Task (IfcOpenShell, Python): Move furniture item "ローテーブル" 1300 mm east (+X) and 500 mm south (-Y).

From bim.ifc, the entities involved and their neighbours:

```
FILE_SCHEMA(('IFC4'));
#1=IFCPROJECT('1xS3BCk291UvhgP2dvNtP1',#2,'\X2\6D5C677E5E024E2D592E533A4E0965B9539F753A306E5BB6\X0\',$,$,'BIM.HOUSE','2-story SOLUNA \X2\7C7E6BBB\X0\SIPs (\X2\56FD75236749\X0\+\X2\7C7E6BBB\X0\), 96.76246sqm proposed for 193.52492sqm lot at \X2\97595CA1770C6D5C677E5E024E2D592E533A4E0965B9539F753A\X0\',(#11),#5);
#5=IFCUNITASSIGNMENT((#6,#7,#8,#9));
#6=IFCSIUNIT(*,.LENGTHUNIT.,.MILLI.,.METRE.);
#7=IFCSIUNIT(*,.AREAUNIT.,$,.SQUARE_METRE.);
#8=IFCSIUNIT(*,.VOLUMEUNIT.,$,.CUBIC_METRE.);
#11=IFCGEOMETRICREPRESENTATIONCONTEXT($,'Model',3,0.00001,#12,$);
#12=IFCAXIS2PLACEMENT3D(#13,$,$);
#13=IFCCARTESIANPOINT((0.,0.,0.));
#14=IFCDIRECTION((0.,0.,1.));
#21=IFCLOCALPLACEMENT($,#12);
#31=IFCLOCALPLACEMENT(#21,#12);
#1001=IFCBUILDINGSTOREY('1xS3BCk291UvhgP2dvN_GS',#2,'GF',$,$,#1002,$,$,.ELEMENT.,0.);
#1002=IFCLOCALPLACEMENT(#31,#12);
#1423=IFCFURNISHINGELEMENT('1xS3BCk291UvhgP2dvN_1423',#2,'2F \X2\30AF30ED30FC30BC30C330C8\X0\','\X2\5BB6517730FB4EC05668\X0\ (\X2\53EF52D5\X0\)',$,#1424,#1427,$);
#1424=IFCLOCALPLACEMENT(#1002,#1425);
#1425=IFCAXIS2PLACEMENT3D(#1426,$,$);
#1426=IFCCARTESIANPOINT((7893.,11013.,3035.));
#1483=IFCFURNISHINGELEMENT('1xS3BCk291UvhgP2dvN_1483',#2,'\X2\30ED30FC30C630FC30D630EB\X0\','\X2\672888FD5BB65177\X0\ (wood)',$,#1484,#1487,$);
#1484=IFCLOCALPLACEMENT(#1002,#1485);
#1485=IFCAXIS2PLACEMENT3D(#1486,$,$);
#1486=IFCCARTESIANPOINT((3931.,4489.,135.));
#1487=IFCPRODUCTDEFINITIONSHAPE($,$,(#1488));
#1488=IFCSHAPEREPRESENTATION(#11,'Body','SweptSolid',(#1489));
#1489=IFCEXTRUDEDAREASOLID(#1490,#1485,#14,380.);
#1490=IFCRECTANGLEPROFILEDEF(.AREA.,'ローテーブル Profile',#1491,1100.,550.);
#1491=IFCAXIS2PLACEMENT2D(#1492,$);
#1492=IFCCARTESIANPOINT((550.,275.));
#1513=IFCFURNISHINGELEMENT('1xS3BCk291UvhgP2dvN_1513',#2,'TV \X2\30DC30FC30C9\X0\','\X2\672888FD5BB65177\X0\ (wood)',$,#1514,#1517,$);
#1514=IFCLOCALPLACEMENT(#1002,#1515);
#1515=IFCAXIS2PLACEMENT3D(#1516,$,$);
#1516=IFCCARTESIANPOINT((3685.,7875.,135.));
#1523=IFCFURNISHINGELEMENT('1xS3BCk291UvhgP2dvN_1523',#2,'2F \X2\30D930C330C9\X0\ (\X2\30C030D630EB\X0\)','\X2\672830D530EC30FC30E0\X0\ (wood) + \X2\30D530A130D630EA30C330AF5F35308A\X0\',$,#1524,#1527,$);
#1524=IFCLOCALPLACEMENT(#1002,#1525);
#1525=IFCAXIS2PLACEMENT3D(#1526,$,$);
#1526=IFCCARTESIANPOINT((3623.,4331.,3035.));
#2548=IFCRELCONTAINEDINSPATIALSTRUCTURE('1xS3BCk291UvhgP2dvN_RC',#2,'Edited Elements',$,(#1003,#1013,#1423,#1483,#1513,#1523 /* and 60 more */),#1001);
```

```python
import ifcopenshell
import ifcopenshell.api.geometry
import ifcopenshell.util.placement

model = ifcopenshell.open("bim.ifc")

item = model.by_guid("1xS3BCk291UvhgP2dvN_1483")
matrix = ifcopenshell.util.placement.get_local_placement(item.ObjectPlacement)
matrix[0, 3] += 1300.0
matrix[1, 3] -= 500.0
ifcopenshell.api.geometry.edit_object_placement(model, product=item, matrix=matrix, is_si=False)

print(ifcopenshell.util.placement.get_local_placement(item.ObjectPlacement).round(3) + 0.0)

model.write("bim_rev.ifc")
```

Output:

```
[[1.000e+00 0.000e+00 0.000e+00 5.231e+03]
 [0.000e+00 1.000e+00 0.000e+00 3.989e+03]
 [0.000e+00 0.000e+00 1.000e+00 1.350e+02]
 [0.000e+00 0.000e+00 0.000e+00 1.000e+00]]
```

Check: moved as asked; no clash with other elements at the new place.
